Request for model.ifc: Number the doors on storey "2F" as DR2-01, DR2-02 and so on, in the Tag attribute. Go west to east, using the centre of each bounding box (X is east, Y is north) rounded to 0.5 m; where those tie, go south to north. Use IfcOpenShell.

First a look at what the model holds.

```python
import ifcopenshell
import ifcopenshell.util.element
import ifcopenshell.util.placement

model = ifcopenshell.open("model.ifc")
print(model.schema)
storey = next(s for s in model.by_type("IfcBuildingStorey") if s.Name == "2F")
doors = [e for e in ifcopenshell.util.element.get_decomposition(storey) if e.is_a("IfcDoor")]
for e in sorted(doors, key=lambda e: e.id()):
    origin = ifcopenshell.util.placement.get_local_placement(e.ObjectPlacement)[:3, 3]
    print(e.id(), e.Tag, e.Name, origin.round(2) + 0.0, sep=" | ")
```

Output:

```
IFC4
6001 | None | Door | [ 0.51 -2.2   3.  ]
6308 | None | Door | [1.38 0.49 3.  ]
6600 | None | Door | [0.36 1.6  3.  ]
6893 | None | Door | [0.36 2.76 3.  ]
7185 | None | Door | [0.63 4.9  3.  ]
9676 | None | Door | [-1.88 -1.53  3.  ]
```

```python
import ifcopenshell
import ifcopenshell.geom
import ifcopenshell.util.element
import ifcopenshell.util.shape

model = ifcopenshell.open("model.ifc")
settings = ifcopenshell.geom.settings()
settings.set("use-world-coords", True)


def centre(element):
    shape = ifcopenshell.geom.create_shape(settings, element)
    return ifcopenshell.util.shape.get_bbox_centroid(shape.geometry)


storey = next(s for s in model.by_type("IfcBuildingStorey") if s.Name == "2F")
doors = [e for e in ifcopenshell.util.element.get_decomposition(storey) if e.is_a("IfcDoor")]

# Insertion points can sit at a corner or the storey origin, so sort by the geometry (in metres).
centres = {e: centre(e) for e in doors}
doors.sort(key=lambda e: (round(centres[e][0] / 0.5), centres[e][1]))

for i, e in enumerate(doors, start=1):
    number = f"DR2-{i:02d}"
    e.Tag = number
    print(e.id(), number)

model.write("model_updated.ifc")
```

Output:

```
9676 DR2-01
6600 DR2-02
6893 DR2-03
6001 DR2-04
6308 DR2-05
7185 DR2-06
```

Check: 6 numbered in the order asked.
